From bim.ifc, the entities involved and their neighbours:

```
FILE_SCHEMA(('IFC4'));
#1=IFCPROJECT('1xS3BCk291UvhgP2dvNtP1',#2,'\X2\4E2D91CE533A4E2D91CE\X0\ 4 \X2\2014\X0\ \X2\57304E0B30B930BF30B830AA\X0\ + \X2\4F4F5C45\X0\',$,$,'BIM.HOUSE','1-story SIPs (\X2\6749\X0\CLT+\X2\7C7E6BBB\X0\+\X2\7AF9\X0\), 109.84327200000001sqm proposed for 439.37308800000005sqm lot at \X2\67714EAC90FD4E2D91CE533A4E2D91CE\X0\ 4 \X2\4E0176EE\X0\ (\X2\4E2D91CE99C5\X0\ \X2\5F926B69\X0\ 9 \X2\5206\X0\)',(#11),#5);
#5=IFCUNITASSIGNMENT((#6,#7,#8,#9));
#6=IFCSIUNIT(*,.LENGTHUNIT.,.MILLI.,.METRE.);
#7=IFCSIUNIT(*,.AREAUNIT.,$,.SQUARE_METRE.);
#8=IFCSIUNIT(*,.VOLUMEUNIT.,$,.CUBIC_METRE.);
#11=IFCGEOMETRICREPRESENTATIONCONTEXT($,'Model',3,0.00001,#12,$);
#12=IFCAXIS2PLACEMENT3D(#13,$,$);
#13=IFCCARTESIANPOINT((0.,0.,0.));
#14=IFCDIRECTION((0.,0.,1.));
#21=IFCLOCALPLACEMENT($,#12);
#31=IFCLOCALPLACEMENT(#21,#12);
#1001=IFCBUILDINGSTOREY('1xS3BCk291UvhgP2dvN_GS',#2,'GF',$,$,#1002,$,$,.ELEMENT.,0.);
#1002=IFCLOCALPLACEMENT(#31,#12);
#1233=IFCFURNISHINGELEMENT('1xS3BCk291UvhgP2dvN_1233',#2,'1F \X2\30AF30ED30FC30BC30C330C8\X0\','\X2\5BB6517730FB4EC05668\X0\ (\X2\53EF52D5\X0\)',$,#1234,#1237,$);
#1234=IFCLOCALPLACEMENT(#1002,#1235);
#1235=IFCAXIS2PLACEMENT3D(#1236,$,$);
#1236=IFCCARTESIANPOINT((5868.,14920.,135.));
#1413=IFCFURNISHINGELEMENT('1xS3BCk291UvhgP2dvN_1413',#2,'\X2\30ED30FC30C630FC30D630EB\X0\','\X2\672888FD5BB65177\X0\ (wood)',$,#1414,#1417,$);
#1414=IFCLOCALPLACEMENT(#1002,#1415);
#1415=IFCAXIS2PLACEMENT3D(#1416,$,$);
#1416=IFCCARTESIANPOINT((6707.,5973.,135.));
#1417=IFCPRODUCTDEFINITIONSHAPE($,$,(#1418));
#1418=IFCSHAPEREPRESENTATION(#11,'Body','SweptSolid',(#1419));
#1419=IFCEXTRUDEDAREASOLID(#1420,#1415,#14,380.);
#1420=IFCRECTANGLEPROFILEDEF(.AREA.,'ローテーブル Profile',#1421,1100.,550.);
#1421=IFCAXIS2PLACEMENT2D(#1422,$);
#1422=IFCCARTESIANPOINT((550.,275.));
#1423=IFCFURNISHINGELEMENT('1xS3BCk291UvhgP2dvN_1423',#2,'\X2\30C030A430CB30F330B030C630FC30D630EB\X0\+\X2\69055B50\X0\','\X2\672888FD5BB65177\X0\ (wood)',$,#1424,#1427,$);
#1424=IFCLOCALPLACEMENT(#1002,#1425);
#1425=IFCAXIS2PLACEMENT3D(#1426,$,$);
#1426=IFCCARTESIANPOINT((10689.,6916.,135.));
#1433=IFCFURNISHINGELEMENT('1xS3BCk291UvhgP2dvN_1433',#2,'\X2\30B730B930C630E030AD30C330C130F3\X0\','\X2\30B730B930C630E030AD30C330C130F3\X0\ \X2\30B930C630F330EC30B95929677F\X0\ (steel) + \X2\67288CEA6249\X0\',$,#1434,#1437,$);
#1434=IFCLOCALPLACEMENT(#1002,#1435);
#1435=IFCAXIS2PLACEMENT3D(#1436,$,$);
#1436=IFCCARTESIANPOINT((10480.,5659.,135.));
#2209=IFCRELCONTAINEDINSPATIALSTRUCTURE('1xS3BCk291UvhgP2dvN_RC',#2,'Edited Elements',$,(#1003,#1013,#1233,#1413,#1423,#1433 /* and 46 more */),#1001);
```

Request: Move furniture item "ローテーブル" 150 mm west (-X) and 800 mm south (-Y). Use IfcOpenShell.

```python
import ifcopenshell
import ifcopenshell.api.geometry
import ifcopenshell.util.placement
import ifcopenshell.util.unit

model = ifcopenshell.open("bim.ifc")
unit_scale = ifcopenshell.util.unit.calculate_unit_scale(model)

item = model.by_guid("1xS3BCk291UvhgP2dvN_1413")
matrix = ifcopenshell.util.placement.get_local_placement(item.ObjectPlacement)
matrix[0, 3] -= 0.15 / unit_scale
matrix[1, 3] -= 0.8 / unit_scale
ifcopenshell.api.geometry.edit_object_placement(model, product=item, matrix=matrix, is_si=False)

print(ifcopenshell.util.placement.get_local_placement(item.ObjectPlacement).round(3) + 0.0)

model.write("bim_updated.ifc")
```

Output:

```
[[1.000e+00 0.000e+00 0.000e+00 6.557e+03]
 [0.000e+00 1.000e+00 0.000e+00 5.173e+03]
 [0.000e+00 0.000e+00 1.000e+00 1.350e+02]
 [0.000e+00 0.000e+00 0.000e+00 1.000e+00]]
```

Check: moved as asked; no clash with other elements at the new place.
